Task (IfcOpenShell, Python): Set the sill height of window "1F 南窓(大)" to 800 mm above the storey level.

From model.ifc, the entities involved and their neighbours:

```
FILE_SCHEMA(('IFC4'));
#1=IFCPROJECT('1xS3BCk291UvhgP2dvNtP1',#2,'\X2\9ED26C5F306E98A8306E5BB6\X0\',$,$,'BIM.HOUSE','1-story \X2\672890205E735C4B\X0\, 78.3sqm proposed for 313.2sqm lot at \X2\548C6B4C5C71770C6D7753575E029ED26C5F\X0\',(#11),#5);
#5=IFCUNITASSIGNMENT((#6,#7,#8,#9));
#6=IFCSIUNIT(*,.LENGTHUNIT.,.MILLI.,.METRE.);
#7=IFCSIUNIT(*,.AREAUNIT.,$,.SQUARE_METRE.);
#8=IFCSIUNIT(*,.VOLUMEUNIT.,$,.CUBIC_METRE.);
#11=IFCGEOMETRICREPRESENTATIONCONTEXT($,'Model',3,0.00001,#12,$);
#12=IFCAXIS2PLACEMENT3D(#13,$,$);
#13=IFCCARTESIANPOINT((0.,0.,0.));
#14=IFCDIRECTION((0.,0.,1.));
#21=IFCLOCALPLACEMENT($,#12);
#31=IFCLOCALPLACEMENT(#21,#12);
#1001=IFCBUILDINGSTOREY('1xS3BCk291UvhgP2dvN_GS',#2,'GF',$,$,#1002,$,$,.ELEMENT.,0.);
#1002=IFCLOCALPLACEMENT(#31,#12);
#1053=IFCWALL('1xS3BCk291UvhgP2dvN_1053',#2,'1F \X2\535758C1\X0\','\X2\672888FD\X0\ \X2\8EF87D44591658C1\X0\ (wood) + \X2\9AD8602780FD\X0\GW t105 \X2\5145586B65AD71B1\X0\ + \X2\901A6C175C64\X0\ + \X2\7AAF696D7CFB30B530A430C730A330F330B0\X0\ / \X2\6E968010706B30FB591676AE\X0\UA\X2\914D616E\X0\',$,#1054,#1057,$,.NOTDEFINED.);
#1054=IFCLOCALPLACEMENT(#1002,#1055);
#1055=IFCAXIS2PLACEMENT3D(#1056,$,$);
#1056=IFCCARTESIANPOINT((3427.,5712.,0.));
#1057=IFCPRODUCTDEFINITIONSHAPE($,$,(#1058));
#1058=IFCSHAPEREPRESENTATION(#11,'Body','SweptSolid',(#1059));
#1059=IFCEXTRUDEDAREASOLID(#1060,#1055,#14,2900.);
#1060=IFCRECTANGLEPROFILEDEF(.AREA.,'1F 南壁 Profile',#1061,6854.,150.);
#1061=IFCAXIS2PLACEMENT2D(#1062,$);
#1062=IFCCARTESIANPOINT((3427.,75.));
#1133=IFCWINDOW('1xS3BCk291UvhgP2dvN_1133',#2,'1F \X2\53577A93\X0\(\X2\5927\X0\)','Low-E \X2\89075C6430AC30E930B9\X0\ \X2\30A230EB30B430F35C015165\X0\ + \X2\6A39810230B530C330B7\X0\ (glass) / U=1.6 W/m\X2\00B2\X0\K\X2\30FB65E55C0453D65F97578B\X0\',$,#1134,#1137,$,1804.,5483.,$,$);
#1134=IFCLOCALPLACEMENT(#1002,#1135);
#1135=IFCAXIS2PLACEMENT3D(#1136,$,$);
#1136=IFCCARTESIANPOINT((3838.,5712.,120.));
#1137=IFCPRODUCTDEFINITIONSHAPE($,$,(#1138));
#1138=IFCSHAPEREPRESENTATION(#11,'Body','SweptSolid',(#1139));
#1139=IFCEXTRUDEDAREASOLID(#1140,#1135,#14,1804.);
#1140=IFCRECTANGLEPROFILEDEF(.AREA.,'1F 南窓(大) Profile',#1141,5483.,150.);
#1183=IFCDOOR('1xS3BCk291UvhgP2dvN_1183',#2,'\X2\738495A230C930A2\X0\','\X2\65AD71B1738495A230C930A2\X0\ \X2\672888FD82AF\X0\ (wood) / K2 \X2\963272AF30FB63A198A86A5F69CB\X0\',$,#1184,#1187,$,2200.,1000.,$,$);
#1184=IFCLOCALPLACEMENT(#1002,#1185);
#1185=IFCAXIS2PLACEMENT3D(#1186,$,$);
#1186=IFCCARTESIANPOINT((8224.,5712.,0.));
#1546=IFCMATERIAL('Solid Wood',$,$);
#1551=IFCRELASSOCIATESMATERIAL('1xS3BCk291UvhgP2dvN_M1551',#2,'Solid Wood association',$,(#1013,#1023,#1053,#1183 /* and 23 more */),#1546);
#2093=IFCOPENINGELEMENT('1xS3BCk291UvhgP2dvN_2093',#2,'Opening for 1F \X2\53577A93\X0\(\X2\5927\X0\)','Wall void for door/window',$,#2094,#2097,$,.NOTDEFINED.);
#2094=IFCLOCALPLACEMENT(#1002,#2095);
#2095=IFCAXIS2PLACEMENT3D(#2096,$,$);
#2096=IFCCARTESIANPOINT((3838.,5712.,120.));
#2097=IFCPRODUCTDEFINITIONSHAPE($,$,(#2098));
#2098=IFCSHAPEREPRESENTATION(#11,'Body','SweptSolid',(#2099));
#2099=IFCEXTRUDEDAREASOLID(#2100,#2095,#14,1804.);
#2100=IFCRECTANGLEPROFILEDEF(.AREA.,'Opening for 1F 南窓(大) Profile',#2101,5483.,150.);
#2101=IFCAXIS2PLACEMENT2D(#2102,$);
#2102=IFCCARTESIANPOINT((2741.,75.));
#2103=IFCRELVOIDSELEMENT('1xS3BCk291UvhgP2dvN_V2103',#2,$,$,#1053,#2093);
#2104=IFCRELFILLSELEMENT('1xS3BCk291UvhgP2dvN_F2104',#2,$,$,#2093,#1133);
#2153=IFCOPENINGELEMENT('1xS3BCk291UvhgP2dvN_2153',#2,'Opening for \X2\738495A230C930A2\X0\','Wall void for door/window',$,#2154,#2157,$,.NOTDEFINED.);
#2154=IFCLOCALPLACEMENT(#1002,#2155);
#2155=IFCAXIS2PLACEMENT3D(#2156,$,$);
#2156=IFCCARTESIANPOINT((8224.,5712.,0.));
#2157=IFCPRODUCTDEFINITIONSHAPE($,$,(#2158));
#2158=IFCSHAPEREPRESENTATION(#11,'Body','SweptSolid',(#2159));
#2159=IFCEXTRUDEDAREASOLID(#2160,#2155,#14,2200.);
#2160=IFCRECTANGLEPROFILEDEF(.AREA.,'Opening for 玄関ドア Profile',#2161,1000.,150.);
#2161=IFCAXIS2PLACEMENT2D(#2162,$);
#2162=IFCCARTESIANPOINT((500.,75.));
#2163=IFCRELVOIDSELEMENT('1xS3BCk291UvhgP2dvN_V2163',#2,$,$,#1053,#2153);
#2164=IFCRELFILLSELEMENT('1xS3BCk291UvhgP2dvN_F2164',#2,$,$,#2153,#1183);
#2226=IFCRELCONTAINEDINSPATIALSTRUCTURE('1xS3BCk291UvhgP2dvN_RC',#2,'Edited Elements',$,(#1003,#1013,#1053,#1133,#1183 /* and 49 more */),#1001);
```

```python
import numpy as np
import ifcopenshell
import ifcopenshell.api.geometry
import ifcopenshell.geom
import ifcopenshell.util.element
import ifcopenshell.util.placement
import ifcopenshell.util.shape
import ifcopenshell.util.unit

model = ifcopenshell.open("model.ifc")
unit_scale = ifcopenshell.util.unit.calculate_unit_scale(model)

window = model.by_guid("1xS3BCk291UvhgP2dvN_1133")
opening = window.FillsVoids[0].RelatingOpeningElement
storey = ifcopenshell.util.element.get_container(window, ifc_class="IfcBuildingStorey")
level = ifcopenshell.util.placement.get_local_placement(storey.ObjectPlacement)[2, 3]

# The opening's origin need not be at the sill, so measure its lowest point.
shape = ifcopenshell.geom.create_shape(ifcopenshell.geom.settings(), opening)
bottom = ifcopenshell.util.shape.get_shape_bottom_elevation(shape, shape.geometry) / unit_scale
dz = level + 0.8 / unit_scale - bottom

shift = np.array([0.0, 0.0, dz])
# The window is not placed relative to its opening, so move both.
for product in (opening, window):
    matrix = ifcopenshell.util.placement.get_local_placement(product.ObjectPlacement)
    matrix[:3, 3] += shift
    ifcopenshell.api.geometry.edit_object_placement(model, product=product, matrix=matrix, is_si=False)

print(f"moved by {dz * unit_scale:+.3f} m")

model.write("model_edited.ifc")
```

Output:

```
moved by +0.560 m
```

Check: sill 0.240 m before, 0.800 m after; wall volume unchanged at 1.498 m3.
